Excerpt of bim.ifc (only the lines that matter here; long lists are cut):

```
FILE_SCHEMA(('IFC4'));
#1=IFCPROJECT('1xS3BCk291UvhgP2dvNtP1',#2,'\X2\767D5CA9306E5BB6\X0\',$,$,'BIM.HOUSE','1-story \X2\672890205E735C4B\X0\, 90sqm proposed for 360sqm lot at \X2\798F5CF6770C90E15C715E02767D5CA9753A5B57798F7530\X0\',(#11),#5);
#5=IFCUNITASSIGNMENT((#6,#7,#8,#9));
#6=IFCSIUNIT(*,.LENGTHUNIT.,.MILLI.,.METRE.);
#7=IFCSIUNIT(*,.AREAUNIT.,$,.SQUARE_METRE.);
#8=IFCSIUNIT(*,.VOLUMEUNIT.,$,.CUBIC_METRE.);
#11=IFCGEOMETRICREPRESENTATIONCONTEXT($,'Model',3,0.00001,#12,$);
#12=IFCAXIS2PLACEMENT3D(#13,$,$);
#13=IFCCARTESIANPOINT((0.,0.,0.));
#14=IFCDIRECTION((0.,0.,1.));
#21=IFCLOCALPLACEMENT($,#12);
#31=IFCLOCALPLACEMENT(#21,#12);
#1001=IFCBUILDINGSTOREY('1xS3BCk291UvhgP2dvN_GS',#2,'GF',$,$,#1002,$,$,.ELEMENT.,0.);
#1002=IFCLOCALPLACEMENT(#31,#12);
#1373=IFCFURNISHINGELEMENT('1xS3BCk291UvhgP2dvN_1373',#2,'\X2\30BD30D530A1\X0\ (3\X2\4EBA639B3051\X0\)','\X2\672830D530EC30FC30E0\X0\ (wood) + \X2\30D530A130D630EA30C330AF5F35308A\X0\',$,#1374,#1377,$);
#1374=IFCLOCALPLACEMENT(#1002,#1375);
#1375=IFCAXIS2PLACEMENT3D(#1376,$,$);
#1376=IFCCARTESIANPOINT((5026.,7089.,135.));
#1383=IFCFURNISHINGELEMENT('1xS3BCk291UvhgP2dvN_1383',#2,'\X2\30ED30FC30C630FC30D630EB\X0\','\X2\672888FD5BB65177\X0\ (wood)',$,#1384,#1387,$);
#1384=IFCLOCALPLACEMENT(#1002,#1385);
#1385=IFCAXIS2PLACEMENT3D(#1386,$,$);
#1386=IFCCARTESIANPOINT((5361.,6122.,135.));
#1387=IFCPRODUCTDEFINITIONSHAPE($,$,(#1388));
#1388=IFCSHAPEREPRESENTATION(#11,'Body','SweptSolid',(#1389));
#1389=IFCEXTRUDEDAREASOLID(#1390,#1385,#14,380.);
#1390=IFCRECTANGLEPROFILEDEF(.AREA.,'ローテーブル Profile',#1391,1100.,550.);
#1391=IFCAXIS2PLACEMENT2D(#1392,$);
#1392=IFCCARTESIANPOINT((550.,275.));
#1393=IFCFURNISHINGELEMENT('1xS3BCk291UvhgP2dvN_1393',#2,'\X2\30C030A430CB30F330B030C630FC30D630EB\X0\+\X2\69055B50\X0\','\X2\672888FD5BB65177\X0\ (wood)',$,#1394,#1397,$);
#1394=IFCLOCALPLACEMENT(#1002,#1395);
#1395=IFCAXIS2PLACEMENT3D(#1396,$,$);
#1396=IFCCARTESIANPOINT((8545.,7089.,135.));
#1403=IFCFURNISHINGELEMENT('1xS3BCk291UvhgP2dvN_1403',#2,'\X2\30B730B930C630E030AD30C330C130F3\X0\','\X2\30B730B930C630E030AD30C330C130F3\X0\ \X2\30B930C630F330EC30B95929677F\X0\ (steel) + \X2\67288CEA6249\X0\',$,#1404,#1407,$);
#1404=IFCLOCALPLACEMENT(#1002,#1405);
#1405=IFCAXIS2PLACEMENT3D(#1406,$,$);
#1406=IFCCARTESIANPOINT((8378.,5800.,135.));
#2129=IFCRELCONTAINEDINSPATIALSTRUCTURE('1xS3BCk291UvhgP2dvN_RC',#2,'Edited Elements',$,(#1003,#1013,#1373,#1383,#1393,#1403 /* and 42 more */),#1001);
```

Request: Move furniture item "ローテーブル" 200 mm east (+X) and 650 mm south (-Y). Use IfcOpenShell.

```python
import ifcopenshell
import ifcopenshell.api.geometry
import ifcopenshell.util.placement
import ifcopenshell.util.unit

model = ifcopenshell.open("bim.ifc")
unit_scale = ifcopenshell.util.unit.calculate_unit_scale(model)

item = model.by_guid("1xS3BCk291UvhgP2dvN_1383")
matrix = ifcopenshell.util.placement.get_local_placement(item.ObjectPlacement)
matrix[0, 3] += 0.2 / unit_scale
matrix[1, 3] -= 0.65 / unit_scale
ifcopenshell.api.geometry.edit_object_placement(model, product=item, matrix=matrix, is_si=False)

print(ifcopenshell.util.placement.get_local_placement(item.ObjectPlacement).round(3) + 0.0)

model.write("bim_updated.ifc")
```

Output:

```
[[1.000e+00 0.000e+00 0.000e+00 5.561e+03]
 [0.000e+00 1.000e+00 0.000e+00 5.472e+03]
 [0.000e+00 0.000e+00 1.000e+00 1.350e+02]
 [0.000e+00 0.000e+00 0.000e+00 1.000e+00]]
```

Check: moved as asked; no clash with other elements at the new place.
